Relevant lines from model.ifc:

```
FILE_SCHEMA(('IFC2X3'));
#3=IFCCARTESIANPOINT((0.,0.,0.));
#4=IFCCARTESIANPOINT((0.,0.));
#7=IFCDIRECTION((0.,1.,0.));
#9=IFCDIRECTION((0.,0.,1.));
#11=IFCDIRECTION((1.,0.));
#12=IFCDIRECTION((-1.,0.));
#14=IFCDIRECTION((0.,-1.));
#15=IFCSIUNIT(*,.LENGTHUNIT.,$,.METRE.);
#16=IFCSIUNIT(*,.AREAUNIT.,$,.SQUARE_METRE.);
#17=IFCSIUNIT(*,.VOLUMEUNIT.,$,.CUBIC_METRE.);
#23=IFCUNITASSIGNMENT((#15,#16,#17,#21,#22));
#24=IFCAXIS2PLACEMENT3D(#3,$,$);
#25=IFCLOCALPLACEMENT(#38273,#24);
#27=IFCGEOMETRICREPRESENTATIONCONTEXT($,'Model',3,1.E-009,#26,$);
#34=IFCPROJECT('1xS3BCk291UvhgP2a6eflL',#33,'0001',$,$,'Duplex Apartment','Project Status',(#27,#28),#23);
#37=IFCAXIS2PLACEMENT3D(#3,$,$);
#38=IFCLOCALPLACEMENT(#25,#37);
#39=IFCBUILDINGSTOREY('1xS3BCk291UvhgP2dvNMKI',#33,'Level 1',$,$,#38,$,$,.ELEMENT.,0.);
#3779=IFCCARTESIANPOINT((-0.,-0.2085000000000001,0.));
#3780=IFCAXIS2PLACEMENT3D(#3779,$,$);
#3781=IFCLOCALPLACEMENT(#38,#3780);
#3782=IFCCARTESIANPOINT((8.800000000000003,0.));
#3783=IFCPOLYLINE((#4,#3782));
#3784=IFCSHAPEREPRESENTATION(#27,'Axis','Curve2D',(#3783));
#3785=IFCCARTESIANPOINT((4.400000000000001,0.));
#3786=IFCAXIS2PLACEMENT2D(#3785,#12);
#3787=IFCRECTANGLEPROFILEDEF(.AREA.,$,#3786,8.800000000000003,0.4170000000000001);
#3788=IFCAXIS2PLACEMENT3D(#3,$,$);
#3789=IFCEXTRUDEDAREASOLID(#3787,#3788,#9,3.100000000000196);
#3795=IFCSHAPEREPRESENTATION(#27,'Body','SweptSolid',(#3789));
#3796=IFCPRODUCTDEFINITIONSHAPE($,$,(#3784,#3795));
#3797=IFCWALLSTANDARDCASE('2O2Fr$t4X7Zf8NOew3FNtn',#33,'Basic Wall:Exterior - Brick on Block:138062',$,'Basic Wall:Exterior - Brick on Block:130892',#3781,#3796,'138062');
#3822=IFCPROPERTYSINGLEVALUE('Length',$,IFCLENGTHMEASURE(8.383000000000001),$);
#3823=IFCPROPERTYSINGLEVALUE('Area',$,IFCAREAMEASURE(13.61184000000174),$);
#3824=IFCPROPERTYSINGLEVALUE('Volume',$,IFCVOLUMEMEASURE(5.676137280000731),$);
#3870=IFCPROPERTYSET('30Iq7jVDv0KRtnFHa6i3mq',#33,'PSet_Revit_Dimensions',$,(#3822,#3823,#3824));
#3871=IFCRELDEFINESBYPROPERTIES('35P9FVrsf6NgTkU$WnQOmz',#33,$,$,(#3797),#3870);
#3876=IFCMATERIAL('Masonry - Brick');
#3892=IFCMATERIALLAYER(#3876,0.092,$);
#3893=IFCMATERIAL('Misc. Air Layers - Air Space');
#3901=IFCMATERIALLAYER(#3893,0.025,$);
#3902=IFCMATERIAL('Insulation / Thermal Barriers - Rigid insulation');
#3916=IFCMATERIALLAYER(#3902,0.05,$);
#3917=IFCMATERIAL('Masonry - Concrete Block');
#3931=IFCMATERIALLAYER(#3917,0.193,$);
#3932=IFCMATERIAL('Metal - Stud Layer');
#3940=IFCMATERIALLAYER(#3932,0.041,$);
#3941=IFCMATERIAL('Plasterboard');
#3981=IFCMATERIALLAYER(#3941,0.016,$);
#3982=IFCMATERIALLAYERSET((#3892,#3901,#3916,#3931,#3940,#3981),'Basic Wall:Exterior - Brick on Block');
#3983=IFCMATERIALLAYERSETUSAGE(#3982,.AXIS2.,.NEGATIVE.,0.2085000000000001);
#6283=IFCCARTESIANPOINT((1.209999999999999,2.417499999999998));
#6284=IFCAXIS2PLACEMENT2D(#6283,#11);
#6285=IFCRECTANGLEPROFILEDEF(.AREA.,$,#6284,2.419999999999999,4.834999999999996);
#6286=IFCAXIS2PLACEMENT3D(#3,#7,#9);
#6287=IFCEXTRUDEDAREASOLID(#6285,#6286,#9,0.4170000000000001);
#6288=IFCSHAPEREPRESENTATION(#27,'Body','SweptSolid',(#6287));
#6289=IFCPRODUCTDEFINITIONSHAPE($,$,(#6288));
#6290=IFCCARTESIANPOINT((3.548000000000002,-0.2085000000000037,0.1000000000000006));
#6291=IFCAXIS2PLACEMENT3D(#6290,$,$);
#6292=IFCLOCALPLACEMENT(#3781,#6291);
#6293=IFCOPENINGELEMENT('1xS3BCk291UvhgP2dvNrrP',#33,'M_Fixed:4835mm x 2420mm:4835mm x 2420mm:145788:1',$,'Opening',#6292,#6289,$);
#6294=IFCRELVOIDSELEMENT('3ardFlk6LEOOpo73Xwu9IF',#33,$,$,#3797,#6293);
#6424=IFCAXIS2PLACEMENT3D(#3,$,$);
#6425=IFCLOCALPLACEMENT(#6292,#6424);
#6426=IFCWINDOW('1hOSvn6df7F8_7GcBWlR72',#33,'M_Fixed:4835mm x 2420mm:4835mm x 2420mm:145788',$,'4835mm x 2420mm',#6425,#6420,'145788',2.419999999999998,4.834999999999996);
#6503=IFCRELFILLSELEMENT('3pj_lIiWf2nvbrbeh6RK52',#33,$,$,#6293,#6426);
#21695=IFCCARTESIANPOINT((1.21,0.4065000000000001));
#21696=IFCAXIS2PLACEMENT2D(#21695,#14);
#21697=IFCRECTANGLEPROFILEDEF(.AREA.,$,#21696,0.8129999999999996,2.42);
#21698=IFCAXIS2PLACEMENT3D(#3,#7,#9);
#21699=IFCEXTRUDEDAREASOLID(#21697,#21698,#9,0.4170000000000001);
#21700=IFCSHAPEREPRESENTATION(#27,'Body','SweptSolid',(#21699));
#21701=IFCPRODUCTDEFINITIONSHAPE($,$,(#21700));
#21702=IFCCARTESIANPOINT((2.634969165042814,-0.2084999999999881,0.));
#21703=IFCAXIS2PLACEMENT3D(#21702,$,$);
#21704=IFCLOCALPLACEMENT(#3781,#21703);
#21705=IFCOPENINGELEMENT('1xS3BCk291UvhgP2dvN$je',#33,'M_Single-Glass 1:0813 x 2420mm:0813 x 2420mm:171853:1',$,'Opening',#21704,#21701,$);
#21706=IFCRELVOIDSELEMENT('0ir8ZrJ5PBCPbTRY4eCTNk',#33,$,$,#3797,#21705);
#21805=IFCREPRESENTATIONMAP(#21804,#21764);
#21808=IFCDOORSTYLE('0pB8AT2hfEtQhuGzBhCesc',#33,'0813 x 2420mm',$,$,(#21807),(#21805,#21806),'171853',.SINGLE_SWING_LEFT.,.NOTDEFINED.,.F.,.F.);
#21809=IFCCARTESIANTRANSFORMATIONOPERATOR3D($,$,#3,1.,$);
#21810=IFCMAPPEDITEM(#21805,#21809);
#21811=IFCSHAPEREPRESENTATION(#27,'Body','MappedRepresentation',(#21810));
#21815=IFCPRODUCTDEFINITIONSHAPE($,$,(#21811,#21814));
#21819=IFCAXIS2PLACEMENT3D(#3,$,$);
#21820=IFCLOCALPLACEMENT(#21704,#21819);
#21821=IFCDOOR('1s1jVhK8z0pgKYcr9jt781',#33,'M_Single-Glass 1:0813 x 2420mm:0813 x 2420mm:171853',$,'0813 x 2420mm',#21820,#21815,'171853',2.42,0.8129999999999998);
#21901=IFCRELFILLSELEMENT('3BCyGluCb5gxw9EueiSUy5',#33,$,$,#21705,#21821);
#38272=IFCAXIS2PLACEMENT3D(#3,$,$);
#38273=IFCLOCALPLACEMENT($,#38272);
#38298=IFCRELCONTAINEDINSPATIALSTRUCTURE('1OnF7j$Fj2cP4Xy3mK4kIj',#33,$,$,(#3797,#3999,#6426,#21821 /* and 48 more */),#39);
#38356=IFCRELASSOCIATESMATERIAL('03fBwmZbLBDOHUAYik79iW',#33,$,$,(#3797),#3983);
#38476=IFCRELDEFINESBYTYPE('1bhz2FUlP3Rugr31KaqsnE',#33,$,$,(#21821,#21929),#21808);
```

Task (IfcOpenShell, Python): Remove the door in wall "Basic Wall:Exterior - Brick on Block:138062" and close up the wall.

```python
import ifcopenshell
import ifcopenshell.api.feature
import ifcopenshell.api.pset
import ifcopenshell.api.root
import ifcopenshell.geom
import ifcopenshell.util.element
import ifcopenshell.util.shape
import ifcopenshell.util.unit

model = ifcopenshell.open("model.ifc")
area_scale = ifcopenshell.util.unit.calculate_unit_scale(model, "AREAUNIT")
volume_scale = ifcopenshell.util.unit.calculate_unit_scale(model, "VOLUMEUNIT")
settings = ifcopenshell.geom.settings()


def volume(element):
    """Net volume in cubic metres, openings subtracted."""
    shape = ifcopenshell.geom.create_shape(settings, element)
    return ifcopenshell.util.shape.get_volume(shape.geometry)


door = model.by_guid("1s1jVhK8z0pgKYcr9jt781")
opening = door.FillsVoids[0].RelatingOpeningElement
wall = opening.VoidsElements[0].RelatingBuildingElement
before = volume(wall)

ifcopenshell.api.root.remove_product(model, product=door)
ifcopenshell.api.feature.remove_feature(model, feature=opening)

after = volume(wall)
thickness = 0.417  # wall thickness in metres

# Update the wall's stored quantities.
pset = model.by_id(ifcopenshell.util.element.get_pset(wall, "PSet_Revit_Dimensions", should_inherit=False)["id"])
ifcopenshell.api.pset.edit_pset(model, pset=pset, properties={
    "Area": model.create_entity("IfcAreaMeasure", after / thickness / area_scale),
    "Volume": model.create_entity("IfcVolumeMeasure", after / volume_scale),
})

print(f"wall volume {before:.3f} -> {after:.3f} m3")

model.write("model_edited.ifc")
```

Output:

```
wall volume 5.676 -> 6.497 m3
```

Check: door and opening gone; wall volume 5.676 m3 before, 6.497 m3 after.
